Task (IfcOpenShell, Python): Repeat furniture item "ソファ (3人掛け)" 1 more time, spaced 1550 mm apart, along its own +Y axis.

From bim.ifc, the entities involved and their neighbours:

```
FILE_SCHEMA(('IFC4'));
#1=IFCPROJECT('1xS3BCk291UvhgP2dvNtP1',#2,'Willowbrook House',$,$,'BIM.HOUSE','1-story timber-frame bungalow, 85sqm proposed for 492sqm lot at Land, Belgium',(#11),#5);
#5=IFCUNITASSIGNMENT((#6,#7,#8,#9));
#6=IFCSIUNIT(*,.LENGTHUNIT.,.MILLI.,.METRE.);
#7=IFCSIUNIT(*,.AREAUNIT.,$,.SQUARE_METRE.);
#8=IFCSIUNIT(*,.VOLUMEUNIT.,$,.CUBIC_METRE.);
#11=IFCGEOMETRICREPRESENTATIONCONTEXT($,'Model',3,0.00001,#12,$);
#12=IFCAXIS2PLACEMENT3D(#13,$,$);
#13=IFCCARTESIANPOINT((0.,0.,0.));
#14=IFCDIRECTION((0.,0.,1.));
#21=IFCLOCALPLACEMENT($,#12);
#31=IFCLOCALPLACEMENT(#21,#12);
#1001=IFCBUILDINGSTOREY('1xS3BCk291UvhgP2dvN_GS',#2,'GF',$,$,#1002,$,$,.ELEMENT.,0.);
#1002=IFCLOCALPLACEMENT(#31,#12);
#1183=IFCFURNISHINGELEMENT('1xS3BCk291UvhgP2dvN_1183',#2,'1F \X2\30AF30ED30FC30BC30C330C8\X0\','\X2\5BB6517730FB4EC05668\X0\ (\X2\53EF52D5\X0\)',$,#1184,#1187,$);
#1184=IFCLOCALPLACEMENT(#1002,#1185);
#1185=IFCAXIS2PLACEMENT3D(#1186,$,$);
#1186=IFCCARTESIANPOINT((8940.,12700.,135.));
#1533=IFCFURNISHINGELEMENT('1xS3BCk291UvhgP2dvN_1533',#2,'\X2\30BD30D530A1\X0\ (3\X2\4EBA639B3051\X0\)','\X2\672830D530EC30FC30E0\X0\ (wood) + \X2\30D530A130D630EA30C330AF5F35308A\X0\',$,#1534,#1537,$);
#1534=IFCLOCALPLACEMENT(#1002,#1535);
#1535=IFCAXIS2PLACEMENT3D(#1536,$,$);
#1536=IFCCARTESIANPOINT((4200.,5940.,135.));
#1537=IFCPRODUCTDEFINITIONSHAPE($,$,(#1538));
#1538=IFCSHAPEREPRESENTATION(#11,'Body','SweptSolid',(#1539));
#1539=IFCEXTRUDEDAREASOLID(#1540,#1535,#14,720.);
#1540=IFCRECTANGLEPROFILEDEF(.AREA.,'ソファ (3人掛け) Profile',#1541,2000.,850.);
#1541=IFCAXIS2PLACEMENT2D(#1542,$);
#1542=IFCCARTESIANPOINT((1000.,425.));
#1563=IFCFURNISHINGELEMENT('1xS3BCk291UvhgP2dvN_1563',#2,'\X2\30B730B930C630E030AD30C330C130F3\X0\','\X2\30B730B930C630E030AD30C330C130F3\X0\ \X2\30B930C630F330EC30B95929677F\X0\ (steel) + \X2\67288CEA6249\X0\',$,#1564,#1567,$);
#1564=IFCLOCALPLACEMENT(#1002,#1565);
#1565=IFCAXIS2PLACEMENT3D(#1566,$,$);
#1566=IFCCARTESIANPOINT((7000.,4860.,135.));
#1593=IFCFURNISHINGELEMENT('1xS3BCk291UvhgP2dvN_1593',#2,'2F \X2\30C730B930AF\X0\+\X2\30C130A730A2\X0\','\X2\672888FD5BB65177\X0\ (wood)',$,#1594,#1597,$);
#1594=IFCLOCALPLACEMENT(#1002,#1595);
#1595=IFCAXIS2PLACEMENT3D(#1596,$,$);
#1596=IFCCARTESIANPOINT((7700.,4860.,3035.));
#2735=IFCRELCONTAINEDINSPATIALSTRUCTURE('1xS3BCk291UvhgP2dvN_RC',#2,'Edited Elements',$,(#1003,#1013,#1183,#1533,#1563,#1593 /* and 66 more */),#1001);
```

```python
import ifcopenshell
import ifcopenshell.api.geometry
import ifcopenshell.api.root
import ifcopenshell.util.element
import ifcopenshell.util.placement

model = ifcopenshell.open("bim.ifc")


def reuse_history(source, copy):
    """copy_class also copies each property set's owner history, people and application; keep the originals."""
    for rel in copy.IsDefinedBy:
        if rel.is_a("IfcRelDefinesByProperties") and (history := rel.RelatingPropertyDefinition.OwnerHistory):
            rel.RelatingPropertyDefinition.OwnerHistory = source.OwnerHistory
            ifcopenshell.util.element.remove_deep2(model, history)


source = model.by_id(1533)
base = ifcopenshell.util.placement.get_local_placement(source.ObjectPlacement)
step = base[:3, 1] * 1550.0

for i in range(1, 2):
    copy = ifcopenshell.api.root.copy_class(model, product=source)
    copy.Representation = ifcopenshell.util.element.copy_deep(
        model, source.Representation, exclude=["IfcGeometricRepresentationContext", "IfcRepresentationMap"]
    )
    reuse_history(source, copy)
    matrix = base.copy()
    matrix[:3, 3] += i * step
    print("added at", matrix[:3, 3].round(3) + 0.0)
    ifcopenshell.api.geometry.edit_object_placement(model, product=copy, matrix=matrix, is_si=False)

model.write("bim_rev.ifc")
```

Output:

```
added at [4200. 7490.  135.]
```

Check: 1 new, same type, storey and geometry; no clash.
